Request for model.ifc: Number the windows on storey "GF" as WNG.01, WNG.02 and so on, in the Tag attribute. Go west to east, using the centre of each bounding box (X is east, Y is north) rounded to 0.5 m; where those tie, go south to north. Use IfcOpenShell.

First a look at what the model holds.

```python
import ifcopenshell
import ifcopenshell.util.element
import ifcopenshell.util.placement

model = ifcopenshell.open("model.ifc")
print(model.schema)
storey = next(s for s in model.by_type("IfcBuildingStorey") if s.Name == "GF")
windows = [e for e in ifcopenshell.util.element.get_decomposition(storey) if e.is_a("IfcWindow")]
for e in sorted(windows, key=lambda e: e.id()):
    origin = ifcopenshell.util.placement.get_local_placement(e.ObjectPlacement)[:3, 3]
    print(e.id(), e.Tag, e.Name, origin.round(2) + 0.0, sep=" | ")
```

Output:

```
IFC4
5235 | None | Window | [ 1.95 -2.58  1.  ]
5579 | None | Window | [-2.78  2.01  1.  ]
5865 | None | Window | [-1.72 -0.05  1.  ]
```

```python
import ifcopenshell
import ifcopenshell.geom
import ifcopenshell.util.element
import ifcopenshell.util.shape

model = ifcopenshell.open("model.ifc")
settings = ifcopenshell.geom.settings()
settings.set("use-world-coords", True)


def centre(element):
    shape = ifcopenshell.geom.create_shape(settings, element)
    return ifcopenshell.util.shape.get_bbox_centroid(shape.geometry)


storey = next(s for s in model.by_type("IfcBuildingStorey") if s.Name == "GF")
windows = [e for e in ifcopenshell.util.element.get_decomposition(storey) if e.is_a("IfcWindow")]

# Insertion points can sit at a corner or the storey origin, so sort by the geometry (in metres).
centres = {e: centre(e) for e in windows}
windows.sort(key=lambda e: (round(centres[e][0] / 0.5), centres[e][1]))

for i, e in enumerate(windows, start=1):
    number = f"WNG.{i:02d}"
    e.Tag = number
    print(e.id(), number)

model.write("model_edited.ifc")
```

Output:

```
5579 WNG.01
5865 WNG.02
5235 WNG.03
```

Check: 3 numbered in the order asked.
